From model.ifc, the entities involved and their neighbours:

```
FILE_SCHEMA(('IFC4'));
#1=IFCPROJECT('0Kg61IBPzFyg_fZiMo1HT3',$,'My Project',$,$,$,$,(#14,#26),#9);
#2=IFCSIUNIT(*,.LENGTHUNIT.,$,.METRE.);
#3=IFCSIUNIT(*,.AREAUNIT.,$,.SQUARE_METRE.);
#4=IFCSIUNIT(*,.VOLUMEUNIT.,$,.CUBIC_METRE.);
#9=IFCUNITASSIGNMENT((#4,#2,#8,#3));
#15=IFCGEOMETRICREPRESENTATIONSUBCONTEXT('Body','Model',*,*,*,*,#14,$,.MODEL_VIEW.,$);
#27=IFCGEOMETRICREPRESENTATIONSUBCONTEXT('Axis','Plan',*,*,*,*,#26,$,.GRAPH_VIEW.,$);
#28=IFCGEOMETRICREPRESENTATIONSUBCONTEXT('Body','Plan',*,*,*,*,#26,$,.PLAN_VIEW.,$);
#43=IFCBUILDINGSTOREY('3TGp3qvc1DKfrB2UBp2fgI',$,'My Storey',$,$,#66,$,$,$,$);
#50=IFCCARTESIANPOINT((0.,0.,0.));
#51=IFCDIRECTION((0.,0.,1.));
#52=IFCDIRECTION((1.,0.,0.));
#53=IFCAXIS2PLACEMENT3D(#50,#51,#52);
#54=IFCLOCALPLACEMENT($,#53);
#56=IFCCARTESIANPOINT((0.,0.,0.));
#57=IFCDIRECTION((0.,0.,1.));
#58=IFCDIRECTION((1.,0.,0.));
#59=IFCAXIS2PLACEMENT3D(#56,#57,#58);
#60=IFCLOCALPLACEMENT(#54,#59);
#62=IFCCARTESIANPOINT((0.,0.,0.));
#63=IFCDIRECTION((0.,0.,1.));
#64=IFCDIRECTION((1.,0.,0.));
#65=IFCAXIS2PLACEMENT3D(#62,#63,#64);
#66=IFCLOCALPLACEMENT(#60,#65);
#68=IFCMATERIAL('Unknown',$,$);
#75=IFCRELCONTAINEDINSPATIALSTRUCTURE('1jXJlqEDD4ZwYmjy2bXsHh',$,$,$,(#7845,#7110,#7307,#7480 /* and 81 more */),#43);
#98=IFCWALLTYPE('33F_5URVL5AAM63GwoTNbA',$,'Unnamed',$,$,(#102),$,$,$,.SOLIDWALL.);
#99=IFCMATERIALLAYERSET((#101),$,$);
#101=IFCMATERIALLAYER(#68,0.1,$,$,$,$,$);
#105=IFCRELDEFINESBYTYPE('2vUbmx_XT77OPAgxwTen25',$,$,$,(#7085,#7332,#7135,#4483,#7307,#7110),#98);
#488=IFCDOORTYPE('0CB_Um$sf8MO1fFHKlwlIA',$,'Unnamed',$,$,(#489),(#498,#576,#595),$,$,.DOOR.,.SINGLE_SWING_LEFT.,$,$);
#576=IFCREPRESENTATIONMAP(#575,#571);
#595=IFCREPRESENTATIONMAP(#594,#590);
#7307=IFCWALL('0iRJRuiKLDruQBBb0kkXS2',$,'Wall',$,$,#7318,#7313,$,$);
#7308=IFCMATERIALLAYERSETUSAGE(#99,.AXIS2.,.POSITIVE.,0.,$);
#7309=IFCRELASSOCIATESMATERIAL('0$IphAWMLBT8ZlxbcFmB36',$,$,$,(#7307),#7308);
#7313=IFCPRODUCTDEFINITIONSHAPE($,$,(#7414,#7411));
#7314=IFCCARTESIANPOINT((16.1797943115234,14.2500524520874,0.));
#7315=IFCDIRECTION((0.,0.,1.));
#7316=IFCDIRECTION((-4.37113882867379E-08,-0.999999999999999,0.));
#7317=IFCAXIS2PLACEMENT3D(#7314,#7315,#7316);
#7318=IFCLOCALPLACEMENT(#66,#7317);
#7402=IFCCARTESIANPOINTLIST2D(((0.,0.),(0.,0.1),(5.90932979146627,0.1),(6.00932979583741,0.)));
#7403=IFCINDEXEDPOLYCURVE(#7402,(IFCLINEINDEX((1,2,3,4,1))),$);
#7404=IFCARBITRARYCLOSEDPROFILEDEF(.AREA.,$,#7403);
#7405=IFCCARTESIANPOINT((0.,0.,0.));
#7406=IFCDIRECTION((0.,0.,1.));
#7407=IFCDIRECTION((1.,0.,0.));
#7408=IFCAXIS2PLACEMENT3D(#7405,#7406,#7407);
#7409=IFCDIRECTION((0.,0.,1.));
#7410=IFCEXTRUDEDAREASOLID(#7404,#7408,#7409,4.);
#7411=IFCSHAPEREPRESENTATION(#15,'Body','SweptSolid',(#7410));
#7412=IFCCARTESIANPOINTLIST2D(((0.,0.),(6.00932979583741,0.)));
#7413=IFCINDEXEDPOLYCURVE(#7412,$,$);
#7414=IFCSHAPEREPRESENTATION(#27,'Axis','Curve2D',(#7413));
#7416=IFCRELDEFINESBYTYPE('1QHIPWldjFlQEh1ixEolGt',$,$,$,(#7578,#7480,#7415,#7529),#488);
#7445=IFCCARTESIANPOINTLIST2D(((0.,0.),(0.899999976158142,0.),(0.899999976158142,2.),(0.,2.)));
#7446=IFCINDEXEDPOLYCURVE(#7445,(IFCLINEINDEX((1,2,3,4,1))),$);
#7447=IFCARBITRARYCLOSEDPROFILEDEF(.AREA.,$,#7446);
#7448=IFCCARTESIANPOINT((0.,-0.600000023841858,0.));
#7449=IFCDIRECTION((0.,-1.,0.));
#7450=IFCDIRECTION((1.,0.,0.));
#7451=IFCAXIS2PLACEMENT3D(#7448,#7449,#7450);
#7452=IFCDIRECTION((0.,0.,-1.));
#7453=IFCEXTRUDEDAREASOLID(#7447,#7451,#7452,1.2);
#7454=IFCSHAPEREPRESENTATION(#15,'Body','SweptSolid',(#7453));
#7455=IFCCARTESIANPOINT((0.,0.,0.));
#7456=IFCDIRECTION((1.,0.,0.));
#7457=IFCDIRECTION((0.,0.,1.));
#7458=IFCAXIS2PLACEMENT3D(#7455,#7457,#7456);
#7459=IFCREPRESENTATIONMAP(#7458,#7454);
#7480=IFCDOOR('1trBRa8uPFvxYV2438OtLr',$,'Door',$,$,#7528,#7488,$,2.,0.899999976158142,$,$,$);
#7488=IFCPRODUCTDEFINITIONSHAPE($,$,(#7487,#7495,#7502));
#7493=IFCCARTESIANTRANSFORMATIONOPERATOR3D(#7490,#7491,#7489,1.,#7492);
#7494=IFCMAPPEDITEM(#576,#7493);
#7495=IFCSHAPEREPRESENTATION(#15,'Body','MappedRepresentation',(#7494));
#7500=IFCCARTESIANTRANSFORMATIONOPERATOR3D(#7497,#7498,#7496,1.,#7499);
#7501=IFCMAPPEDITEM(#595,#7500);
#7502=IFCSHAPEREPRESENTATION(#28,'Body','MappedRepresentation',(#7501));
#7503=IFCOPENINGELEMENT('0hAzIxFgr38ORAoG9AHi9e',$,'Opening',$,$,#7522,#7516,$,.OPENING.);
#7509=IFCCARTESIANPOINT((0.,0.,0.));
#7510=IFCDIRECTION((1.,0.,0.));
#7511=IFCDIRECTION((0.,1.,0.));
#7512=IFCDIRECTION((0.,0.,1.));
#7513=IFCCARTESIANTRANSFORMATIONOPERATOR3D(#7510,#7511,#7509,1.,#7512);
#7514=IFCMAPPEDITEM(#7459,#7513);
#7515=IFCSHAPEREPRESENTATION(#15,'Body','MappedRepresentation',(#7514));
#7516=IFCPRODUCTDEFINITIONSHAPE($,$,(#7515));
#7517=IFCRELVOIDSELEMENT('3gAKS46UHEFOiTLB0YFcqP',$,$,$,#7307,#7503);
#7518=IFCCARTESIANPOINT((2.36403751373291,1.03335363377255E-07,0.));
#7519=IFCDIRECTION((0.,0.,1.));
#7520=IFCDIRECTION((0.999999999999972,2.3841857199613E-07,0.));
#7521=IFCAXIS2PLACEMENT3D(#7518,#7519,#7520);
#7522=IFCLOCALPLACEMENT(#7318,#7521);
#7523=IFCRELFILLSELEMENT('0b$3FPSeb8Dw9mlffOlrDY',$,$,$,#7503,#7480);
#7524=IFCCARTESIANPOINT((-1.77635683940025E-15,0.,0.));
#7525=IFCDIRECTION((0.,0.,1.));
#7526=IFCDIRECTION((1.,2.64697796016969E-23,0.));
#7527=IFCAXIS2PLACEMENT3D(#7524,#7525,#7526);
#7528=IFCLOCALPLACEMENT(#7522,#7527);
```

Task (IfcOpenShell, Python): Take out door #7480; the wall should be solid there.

```python
import ifcopenshell
import ifcopenshell.api.feature
import ifcopenshell.api.root
import ifcopenshell.geom
import ifcopenshell.util.shape

model = ifcopenshell.open("model.ifc")
settings = ifcopenshell.geom.settings()


def volume(element):
    """Net volume in cubic metres, openings subtracted."""
    shape = ifcopenshell.geom.create_shape(settings, element)
    return ifcopenshell.util.shape.get_volume(shape.geometry)


door = model.by_id(7480)
opening = door.FillsVoids[0].RelatingOpeningElement
wall = opening.VoidsElements[0].RelatingBuildingElement
before = volume(wall)

ifcopenshell.api.root.remove_product(model, product=door)
ifcopenshell.api.feature.remove_feature(model, feature=opening)

after = volume(wall)

print(f"wall volume {before:.3f} -> {after:.3f} m3")

model.write("model_edited.ifc")
```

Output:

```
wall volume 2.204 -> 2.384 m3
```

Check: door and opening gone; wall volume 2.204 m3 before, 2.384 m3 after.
